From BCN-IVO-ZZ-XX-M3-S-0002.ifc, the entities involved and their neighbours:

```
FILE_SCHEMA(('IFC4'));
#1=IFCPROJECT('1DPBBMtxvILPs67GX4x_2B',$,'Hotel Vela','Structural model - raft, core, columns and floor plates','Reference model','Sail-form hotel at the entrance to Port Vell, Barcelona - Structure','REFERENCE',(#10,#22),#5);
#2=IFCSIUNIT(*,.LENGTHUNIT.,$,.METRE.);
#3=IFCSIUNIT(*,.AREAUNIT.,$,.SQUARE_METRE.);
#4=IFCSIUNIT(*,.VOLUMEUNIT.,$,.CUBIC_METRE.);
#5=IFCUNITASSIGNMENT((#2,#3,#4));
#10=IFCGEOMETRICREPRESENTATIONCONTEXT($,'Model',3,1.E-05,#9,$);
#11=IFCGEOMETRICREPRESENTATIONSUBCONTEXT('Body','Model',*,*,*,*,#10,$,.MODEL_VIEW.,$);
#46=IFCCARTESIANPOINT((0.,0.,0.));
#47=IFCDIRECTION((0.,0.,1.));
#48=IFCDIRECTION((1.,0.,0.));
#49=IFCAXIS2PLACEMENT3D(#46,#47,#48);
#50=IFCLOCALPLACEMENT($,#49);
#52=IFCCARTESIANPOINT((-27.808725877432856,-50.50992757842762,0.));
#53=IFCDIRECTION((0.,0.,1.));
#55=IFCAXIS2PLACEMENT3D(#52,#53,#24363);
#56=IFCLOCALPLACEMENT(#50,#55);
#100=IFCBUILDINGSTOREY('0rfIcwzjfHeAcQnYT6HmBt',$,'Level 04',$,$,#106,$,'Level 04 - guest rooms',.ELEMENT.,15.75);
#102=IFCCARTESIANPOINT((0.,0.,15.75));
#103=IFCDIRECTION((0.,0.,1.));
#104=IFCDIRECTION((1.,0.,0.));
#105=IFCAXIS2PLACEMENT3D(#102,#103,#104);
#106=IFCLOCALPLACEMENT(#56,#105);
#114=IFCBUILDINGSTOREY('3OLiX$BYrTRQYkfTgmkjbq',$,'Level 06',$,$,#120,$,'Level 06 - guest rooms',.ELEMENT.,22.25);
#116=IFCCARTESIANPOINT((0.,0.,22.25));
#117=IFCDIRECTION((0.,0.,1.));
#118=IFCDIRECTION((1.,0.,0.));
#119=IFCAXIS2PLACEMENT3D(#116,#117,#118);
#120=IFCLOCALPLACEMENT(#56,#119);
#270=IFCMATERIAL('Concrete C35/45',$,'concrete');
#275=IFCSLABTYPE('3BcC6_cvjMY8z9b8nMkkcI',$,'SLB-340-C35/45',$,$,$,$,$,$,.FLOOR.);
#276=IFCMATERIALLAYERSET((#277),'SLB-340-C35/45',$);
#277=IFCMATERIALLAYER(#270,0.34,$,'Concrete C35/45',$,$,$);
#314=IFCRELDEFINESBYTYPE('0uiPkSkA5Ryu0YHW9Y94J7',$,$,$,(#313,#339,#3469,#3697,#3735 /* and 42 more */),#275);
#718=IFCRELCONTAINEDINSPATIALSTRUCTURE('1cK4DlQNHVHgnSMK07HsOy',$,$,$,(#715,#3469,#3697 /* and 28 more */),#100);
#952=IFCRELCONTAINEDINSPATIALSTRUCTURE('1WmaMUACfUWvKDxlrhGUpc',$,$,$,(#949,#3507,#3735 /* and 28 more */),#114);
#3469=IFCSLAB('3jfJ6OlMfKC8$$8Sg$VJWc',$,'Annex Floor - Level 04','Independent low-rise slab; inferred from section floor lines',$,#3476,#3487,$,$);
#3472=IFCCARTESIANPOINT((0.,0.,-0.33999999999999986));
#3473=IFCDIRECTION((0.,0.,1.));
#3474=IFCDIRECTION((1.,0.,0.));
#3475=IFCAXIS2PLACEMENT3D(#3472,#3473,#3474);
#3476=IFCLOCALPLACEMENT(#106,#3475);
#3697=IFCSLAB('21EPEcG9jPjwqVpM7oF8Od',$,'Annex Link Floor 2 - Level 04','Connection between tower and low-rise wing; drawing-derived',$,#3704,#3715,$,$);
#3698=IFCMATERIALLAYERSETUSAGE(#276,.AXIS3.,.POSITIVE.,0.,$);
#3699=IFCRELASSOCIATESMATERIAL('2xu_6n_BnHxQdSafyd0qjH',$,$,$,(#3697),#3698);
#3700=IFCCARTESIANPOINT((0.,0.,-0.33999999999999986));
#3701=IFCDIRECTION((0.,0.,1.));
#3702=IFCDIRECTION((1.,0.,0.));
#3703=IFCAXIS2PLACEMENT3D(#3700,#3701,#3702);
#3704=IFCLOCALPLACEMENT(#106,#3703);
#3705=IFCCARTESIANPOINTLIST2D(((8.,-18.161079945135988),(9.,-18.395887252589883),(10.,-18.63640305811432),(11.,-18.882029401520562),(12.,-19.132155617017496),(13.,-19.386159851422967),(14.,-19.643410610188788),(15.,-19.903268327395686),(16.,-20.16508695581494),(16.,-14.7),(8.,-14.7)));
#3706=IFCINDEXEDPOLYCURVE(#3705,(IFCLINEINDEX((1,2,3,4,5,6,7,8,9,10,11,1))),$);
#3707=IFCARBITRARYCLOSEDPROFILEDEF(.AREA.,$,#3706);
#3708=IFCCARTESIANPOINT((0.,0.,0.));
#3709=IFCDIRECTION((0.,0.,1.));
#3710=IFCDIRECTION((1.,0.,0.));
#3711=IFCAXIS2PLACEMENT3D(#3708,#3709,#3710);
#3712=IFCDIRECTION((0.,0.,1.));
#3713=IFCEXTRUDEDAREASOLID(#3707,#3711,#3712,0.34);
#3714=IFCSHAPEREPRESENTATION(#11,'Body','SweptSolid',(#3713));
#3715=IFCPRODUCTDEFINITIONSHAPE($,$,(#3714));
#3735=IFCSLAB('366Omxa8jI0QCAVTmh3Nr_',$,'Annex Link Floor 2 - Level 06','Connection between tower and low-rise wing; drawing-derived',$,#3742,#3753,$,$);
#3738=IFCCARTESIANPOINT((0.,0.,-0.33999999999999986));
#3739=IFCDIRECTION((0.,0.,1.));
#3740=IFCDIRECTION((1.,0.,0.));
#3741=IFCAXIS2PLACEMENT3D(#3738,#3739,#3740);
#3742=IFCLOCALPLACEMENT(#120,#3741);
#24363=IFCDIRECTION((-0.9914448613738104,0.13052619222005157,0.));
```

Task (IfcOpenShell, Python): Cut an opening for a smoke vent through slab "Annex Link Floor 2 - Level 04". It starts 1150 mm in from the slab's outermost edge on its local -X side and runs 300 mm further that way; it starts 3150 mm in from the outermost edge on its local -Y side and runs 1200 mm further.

```python
import numpy as np
import ifcopenshell
import ifcopenshell.api.feature
import ifcopenshell.api.geometry
import ifcopenshell.api.root
import ifcopenshell.geom
import ifcopenshell.util.placement
import ifcopenshell.util.representation
import ifcopenshell.util.shape
import ifcopenshell.util.unit

model = ifcopenshell.open("BCN-IVO-ZZ-XX-M3-S-0002.ifc")
unit_scale = ifcopenshell.util.unit.calculate_unit_scale(model)
settings = ifcopenshell.geom.settings()


def volume(element):
    """Net volume in cubic metres, openings subtracted."""
    shape = ifcopenshell.geom.create_shape(settings, element)
    return ifcopenshell.util.shape.get_volume(shape.geometry)


slab = model.by_guid("21EPEcG9jPjwqVpM7oF8Od")
before = volume(slab)

# Extent in the slab's own axes, in metres. The edges named are its -X and -Y sides.
slab_shape = ifcopenshell.geom.create_shape(settings, slab)
vertices = ifcopenshell.util.shape.get_vertices(slab_shape.geometry)
x_min, y_min, bottom = vertices.min(axis=0)
top = vertices[:, 2].max()

opening = ifcopenshell.api.root.create_entity(model, ifc_class="IfcOpeningElement", name="Smoke vent opening", predefined_type="OPENING")
context = ifcopenshell.util.representation.get_context(model, "Model", "Body", "MODEL_VIEW")
width, depth = 0.3, 1.2
outline = [(0.0, 0.0), (width, 0.0), (width, depth), (0.0, depth), (0.0, 0.0)]
# Overshoot both faces by 50 mm so the cut is clean.
shape = ifcopenshell.api.geometry.add_slab_representation(
    model, context=context, depth=top - bottom + 0.1, polyline=outline
)
ifcopenshell.api.geometry.assign_representation(model, product=opening, representation=shape)

matrix = ifcopenshell.util.placement.get_local_placement(slab.ObjectPlacement)
matrix[:, 3] = matrix @ np.append(np.array([x_min + 1.15, y_min + 3.15, bottom - 0.05]) / unit_scale, 1.0)
ifcopenshell.api.geometry.edit_object_placement(model, product=opening, matrix=matrix, is_si=False)
ifcopenshell.api.feature.add_feature(model, feature=opening, element=slab)

after = volume(slab)

print(f"slab volume {before:.3f} -> {after:.3f} m3")

model.write("BCN-IVO-ZZ-XX-M3-S-0002_v2.ifc")
```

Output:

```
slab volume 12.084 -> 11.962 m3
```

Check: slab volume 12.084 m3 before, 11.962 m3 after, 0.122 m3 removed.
